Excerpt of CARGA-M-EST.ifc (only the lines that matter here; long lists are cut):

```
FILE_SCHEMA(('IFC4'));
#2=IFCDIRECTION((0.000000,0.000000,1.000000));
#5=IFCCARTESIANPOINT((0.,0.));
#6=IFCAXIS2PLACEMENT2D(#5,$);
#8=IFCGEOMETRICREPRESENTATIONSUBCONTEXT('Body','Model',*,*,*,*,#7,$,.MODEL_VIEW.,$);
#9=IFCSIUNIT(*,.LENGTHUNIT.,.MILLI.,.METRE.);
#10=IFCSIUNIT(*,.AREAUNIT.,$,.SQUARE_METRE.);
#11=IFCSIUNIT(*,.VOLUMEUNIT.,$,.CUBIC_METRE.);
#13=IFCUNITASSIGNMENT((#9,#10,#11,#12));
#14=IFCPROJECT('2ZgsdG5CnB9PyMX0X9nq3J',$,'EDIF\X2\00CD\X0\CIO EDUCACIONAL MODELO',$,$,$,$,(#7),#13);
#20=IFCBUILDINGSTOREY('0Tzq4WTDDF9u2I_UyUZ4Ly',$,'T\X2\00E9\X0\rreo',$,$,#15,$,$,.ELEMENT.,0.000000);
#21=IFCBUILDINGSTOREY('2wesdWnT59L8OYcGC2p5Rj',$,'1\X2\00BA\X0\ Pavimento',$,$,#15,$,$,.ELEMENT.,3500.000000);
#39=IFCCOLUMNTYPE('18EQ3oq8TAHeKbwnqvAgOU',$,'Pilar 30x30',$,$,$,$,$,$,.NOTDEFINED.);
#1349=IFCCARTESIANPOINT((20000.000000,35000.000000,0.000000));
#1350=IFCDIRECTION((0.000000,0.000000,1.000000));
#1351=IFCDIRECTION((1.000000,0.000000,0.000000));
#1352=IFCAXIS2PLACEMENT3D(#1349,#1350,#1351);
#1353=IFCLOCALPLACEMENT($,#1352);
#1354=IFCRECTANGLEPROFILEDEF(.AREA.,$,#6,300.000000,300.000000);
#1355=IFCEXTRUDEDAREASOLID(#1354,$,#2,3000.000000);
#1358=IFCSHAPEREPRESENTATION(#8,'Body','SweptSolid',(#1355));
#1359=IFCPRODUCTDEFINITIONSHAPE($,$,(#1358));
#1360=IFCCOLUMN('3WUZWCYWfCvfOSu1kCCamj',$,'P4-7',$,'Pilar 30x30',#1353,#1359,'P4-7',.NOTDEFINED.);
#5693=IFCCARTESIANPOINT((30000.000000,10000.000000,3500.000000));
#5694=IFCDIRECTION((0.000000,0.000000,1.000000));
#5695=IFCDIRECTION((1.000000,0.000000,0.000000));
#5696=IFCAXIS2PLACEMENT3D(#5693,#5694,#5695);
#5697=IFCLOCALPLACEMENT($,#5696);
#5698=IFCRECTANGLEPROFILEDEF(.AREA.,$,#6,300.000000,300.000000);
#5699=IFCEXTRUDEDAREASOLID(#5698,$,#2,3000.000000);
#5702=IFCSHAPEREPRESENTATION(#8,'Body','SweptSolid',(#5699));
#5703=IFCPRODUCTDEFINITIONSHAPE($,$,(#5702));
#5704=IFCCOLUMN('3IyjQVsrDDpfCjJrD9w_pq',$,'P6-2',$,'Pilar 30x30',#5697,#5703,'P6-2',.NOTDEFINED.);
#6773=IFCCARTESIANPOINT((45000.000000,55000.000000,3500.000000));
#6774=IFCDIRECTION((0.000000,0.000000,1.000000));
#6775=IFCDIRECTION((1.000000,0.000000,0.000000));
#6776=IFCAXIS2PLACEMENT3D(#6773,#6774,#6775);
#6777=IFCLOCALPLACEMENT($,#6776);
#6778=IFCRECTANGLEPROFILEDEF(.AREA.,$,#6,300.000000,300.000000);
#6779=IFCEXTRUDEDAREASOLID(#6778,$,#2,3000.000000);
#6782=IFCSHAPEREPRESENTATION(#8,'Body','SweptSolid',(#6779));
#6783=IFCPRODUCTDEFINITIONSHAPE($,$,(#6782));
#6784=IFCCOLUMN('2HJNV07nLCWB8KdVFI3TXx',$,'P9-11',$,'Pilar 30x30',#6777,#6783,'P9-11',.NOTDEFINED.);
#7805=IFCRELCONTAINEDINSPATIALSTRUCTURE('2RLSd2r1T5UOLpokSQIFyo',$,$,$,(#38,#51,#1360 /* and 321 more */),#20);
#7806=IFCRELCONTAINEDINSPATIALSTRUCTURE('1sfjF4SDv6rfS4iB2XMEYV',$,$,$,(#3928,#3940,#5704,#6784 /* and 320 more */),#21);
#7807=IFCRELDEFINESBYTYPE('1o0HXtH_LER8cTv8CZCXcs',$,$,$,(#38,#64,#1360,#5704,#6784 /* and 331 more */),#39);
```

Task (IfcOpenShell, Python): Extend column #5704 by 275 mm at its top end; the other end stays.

```python
import ifcopenshell
import ifcopenshell.util.representation

model = ifcopenshell.open("CARGA-M-EST.ifc")

member = model.by_guid("3IyjQVsrDDpfCjJrD9w_pq")
change = 275.0

# The extrusion runs towards the end named, so only its depth changes.
body = ifcopenshell.util.representation.get_representation(member, "Model", "Body")
solid = body.Items[0]
old_length = solid.Depth
solid.Depth += change

print(f"length {old_length:g} -> {solid.Depth:g}")

model.write("CARGA-M-EST_rev.ifc")
```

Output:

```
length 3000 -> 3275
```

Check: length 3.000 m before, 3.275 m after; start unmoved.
